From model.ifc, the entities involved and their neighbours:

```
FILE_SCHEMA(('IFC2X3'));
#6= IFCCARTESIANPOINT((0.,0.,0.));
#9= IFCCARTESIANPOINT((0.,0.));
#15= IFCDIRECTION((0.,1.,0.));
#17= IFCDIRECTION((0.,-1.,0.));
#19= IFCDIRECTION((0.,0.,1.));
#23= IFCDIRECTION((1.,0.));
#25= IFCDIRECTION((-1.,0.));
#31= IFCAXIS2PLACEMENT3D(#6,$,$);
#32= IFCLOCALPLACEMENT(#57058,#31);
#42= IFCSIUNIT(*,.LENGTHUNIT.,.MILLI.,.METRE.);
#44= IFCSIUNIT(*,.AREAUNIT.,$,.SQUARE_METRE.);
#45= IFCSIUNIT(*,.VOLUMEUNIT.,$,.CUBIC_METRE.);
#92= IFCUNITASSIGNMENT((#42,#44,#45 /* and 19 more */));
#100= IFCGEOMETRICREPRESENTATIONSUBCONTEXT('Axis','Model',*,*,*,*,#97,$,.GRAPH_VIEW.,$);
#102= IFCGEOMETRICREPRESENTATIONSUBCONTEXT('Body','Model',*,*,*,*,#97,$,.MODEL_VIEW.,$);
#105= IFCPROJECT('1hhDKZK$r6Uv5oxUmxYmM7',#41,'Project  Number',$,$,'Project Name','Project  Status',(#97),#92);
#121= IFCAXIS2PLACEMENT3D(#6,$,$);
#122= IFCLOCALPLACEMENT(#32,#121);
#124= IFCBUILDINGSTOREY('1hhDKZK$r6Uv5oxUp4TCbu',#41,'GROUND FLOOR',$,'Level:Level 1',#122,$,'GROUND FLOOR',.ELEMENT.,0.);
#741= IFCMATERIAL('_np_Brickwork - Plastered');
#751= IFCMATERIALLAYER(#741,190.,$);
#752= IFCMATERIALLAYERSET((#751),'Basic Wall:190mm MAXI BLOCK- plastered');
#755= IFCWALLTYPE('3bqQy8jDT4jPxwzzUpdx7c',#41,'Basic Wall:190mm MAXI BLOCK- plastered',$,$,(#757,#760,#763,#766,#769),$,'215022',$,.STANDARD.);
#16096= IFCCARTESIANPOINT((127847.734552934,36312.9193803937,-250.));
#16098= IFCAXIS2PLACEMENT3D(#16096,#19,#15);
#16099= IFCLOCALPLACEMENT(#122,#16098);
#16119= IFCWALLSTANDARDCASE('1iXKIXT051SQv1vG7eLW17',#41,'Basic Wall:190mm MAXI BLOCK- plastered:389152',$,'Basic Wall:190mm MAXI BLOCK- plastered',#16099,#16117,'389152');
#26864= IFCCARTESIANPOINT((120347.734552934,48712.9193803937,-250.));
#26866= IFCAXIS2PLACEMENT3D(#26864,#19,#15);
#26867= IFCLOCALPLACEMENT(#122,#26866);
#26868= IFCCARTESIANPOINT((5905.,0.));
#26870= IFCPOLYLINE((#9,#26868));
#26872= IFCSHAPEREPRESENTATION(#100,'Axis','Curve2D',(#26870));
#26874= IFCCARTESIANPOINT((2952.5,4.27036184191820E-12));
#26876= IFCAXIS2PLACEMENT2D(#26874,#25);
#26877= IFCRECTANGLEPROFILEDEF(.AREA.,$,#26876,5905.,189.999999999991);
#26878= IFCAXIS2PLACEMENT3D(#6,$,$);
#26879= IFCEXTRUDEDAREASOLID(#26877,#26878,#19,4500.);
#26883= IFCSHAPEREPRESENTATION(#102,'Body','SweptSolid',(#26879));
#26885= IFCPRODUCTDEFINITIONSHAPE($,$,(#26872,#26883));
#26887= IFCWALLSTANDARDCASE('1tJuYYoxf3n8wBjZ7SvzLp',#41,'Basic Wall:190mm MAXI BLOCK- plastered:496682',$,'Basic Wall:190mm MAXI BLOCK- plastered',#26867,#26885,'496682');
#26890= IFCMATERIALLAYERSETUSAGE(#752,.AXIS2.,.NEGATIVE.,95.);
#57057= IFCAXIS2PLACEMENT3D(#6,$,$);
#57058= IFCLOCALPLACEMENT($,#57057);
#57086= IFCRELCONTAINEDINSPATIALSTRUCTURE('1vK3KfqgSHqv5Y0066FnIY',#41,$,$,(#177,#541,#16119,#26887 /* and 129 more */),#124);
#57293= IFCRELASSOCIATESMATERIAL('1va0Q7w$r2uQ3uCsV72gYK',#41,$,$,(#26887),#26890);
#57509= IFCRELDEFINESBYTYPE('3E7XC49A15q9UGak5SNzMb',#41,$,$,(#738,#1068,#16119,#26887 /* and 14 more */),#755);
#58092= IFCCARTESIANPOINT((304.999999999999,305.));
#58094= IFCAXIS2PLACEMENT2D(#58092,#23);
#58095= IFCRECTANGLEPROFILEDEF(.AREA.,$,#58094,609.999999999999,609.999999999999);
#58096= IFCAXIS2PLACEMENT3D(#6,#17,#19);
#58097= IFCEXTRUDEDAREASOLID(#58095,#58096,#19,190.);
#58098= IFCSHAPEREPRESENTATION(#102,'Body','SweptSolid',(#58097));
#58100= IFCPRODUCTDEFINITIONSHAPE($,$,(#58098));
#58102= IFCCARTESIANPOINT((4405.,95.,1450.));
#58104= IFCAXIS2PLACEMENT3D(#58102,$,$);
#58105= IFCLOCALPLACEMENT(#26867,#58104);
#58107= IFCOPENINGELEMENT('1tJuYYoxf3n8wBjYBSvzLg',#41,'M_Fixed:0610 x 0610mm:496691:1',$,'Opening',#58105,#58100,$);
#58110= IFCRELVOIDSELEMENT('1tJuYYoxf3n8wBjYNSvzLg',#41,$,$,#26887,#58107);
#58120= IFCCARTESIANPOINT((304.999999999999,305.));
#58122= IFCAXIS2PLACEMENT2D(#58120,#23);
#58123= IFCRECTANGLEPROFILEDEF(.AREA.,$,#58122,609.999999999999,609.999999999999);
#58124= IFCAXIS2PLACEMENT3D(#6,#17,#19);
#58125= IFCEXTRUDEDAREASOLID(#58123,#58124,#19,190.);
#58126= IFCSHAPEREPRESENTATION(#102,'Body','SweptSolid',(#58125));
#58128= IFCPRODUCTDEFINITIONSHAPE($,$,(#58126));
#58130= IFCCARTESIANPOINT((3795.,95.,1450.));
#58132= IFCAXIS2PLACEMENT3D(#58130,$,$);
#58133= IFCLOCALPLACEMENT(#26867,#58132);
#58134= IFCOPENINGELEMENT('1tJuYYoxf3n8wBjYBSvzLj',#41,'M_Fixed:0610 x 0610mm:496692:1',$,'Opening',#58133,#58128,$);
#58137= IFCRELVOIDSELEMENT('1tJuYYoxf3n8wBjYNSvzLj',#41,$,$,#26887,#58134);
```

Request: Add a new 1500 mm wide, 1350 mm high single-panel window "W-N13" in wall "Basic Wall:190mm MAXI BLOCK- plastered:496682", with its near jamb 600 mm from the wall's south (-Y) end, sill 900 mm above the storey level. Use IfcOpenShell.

```python
import numpy as np
import ifcopenshell
import ifcopenshell.api.feature
import ifcopenshell.api.geometry
import ifcopenshell.api.root
import ifcopenshell.api.spatial
import ifcopenshell.api.type
import ifcopenshell.geom
import ifcopenshell.util.element
import ifcopenshell.util.placement
import ifcopenshell.util.representation
import ifcopenshell.util.shape
import ifcopenshell.util.unit

model = ifcopenshell.open("model.ifc")
unit_scale = ifcopenshell.util.unit.calculate_unit_scale(model)
settings = ifcopenshell.geom.settings()


def volume(element):
    """Net volume in cubic metres, openings subtracted."""
    shape = ifcopenshell.geom.create_shape(settings, element)
    return ifcopenshell.util.shape.get_volume(shape.geometry)


wall = model.by_id(26887)
storey = ifcopenshell.util.element.get_container(wall, ifc_class="IfcBuildingStorey")
context = ifcopenshell.util.representation.get_context(model, "Model", "Body", "MODEL_VIEW")
before = volume(wall)

width, height, from_end, sill = 1.5, 1.35, 0.6, 0.9  # metres

# The wall runs along its own X axis, and the end named is its -X end.
wall_shape = ifcopenshell.geom.create_shape(settings, wall)
x, y, z = ifcopenshell.util.shape.get_vertices(wall_shape.geometry).T
start = x.min() + from_end
face, thickness = float(y.min()), float(y.max() - y.min())
wall_matrix = ifcopenshell.util.placement.get_local_placement(wall.ObjectPlacement)
level = ifcopenshell.util.placement.get_local_placement(storey.ObjectPlacement)[2, 3]


def in_wall(x, y):
    """Placement at x, y metres in the wall's axes, at sill height."""
    matrix = wall_matrix.copy()
    matrix[:, 3] = wall_matrix @ np.array([x / unit_scale, y / unit_scale, 0.0, 1.0])
    matrix[2, 3] = level + sill / unit_scale
    return matrix


# Opening: a box that overshoots both wall faces by 50 mm.
opening = ifcopenshell.api.root.create_entity(model, ifc_class="IfcOpeningElement")
box = ifcopenshell.api.geometry.add_wall_representation(
    model, context=context, length=width, height=height, thickness=thickness + 0.1
)
ifcopenshell.api.geometry.assign_representation(model, product=opening, representation=box)
ifcopenshell.api.geometry.edit_object_placement(model, product=opening, matrix=in_wall(start, face - 0.05), is_si=False)
ifcopenshell.api.feature.add_feature(model, feature=opening, element=wall)

window = ifcopenshell.api.root.create_entity(model, ifc_class="IfcWindow", name="W-N13")
window.OverallWidth, window.OverallHeight = width / unit_scale, height / unit_scale
body = ifcopenshell.api.geometry.add_window_representation(
    model,
    context=context,
    overall_width=window.OverallWidth,
    overall_height=window.OverallHeight,
    partition_type="SINGLE_PANEL",
)
ifcopenshell.api.geometry.assign_representation(model, product=window, representation=body)
ifcopenshell.api.spatial.assign_container(model, products=[window], relating_structure=storey)
fills = ifcopenshell.api.feature.add_filling(model, opening=opening, element=window)
fills.OwnerHistory = window.OwnerHistory  # required in IFC2X3

# IFC2X3 keeps the operation on the window style.
style = ifcopenshell.api.root.create_entity(model, ifc_class="IfcWindowStyle", name="W-N13")
style.OperationType, style.ConstructionType = "SINGLE_PANEL", "NOTDEFINED"
style.ParameterTakesPrecedence = style.Sizeable = False
ifcopenshell.api.type.assign_type(model, related_objects=[window], relating_type=style)

# Centre the window in the wall's thickness.
ifcopenshell.api.geometry.edit_object_placement(model, product=window, matrix=in_wall(start, face), is_si=False)
window_shape = ifcopenshell.geom.create_shape(settings, window)
depth = ifcopenshell.util.shape.get_vertices(window_shape.geometry)[:, 1]
offset = face + thickness / 2 - (depth.min() + depth.max()) / 2
ifcopenshell.api.geometry.edit_object_placement(model, product=window, matrix=in_wall(start, offset), is_si=False)

after = volume(wall)

print(f"wall volume {before:.3f} -> {after:.3f} m3")

model.write("model_rev.ifc")
```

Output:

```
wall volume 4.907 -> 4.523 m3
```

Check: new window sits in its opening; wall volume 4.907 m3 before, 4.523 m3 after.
